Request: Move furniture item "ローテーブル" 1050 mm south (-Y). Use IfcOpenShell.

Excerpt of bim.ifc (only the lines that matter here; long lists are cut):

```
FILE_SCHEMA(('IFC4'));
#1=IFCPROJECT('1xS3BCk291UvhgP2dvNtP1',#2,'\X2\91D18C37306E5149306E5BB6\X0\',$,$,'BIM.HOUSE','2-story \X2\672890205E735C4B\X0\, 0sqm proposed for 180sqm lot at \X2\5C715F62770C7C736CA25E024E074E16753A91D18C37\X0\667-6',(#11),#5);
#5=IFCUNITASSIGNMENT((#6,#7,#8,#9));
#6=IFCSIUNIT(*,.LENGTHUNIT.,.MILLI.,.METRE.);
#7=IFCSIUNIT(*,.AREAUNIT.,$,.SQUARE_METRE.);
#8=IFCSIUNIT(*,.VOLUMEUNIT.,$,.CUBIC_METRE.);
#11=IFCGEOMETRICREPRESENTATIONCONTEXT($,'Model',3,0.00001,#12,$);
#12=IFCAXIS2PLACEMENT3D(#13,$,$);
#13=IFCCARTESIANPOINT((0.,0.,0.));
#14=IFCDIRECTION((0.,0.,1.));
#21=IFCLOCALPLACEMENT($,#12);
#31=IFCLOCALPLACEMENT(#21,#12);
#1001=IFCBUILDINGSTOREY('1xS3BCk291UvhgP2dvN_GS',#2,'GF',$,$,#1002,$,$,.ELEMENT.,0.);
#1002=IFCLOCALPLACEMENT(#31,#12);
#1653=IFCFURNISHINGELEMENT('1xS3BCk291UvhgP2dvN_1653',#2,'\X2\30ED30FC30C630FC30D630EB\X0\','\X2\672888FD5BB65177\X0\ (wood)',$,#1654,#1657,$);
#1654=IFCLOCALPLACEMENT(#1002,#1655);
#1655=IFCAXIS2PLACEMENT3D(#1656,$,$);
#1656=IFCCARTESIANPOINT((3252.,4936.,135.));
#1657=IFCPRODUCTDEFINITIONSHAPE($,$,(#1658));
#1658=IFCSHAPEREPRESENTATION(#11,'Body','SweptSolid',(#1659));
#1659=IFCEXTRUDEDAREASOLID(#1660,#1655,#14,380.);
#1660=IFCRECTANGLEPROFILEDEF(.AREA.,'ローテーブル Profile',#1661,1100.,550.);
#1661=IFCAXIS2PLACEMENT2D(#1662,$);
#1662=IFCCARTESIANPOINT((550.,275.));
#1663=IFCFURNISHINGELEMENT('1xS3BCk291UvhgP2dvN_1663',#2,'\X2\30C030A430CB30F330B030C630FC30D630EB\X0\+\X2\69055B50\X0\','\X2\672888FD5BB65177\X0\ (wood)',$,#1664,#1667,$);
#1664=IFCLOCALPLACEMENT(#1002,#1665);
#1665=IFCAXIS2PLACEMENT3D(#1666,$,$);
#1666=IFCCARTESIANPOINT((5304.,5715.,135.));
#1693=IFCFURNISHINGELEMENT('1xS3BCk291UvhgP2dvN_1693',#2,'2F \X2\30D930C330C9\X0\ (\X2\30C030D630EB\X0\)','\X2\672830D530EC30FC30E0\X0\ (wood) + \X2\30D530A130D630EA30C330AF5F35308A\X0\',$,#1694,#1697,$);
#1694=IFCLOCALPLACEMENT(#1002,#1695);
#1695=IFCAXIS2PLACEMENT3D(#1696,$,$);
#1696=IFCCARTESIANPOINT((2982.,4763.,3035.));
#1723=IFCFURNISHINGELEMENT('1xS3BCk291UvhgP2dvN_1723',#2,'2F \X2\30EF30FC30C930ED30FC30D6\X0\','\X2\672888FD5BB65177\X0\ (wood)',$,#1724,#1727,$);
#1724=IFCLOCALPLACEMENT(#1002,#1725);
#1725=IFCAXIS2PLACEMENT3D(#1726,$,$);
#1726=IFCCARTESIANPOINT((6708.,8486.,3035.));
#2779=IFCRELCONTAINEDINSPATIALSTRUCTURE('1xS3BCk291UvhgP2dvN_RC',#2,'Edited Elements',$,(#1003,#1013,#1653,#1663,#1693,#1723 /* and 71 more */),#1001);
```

```python
import ifcopenshell
import ifcopenshell.api.geometry
import ifcopenshell.util.placement
import ifcopenshell.util.unit

model = ifcopenshell.open("bim.ifc")
unit_scale = ifcopenshell.util.unit.calculate_unit_scale(model)

item = model.by_guid("1xS3BCk291UvhgP2dvN_1653")
matrix = ifcopenshell.util.placement.get_local_placement(item.ObjectPlacement)
matrix[1, 3] -= 1.05 / unit_scale
ifcopenshell.api.geometry.edit_object_placement(model, product=item, matrix=matrix, is_si=False)

print(ifcopenshell.util.placement.get_local_placement(item.ObjectPlacement).round(3) + 0.0)

model.write("bim_rev.ifc")
```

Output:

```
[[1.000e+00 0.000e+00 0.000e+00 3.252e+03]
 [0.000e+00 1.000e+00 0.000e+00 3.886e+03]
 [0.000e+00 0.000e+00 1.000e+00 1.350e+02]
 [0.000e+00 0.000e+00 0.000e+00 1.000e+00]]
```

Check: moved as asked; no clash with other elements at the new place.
